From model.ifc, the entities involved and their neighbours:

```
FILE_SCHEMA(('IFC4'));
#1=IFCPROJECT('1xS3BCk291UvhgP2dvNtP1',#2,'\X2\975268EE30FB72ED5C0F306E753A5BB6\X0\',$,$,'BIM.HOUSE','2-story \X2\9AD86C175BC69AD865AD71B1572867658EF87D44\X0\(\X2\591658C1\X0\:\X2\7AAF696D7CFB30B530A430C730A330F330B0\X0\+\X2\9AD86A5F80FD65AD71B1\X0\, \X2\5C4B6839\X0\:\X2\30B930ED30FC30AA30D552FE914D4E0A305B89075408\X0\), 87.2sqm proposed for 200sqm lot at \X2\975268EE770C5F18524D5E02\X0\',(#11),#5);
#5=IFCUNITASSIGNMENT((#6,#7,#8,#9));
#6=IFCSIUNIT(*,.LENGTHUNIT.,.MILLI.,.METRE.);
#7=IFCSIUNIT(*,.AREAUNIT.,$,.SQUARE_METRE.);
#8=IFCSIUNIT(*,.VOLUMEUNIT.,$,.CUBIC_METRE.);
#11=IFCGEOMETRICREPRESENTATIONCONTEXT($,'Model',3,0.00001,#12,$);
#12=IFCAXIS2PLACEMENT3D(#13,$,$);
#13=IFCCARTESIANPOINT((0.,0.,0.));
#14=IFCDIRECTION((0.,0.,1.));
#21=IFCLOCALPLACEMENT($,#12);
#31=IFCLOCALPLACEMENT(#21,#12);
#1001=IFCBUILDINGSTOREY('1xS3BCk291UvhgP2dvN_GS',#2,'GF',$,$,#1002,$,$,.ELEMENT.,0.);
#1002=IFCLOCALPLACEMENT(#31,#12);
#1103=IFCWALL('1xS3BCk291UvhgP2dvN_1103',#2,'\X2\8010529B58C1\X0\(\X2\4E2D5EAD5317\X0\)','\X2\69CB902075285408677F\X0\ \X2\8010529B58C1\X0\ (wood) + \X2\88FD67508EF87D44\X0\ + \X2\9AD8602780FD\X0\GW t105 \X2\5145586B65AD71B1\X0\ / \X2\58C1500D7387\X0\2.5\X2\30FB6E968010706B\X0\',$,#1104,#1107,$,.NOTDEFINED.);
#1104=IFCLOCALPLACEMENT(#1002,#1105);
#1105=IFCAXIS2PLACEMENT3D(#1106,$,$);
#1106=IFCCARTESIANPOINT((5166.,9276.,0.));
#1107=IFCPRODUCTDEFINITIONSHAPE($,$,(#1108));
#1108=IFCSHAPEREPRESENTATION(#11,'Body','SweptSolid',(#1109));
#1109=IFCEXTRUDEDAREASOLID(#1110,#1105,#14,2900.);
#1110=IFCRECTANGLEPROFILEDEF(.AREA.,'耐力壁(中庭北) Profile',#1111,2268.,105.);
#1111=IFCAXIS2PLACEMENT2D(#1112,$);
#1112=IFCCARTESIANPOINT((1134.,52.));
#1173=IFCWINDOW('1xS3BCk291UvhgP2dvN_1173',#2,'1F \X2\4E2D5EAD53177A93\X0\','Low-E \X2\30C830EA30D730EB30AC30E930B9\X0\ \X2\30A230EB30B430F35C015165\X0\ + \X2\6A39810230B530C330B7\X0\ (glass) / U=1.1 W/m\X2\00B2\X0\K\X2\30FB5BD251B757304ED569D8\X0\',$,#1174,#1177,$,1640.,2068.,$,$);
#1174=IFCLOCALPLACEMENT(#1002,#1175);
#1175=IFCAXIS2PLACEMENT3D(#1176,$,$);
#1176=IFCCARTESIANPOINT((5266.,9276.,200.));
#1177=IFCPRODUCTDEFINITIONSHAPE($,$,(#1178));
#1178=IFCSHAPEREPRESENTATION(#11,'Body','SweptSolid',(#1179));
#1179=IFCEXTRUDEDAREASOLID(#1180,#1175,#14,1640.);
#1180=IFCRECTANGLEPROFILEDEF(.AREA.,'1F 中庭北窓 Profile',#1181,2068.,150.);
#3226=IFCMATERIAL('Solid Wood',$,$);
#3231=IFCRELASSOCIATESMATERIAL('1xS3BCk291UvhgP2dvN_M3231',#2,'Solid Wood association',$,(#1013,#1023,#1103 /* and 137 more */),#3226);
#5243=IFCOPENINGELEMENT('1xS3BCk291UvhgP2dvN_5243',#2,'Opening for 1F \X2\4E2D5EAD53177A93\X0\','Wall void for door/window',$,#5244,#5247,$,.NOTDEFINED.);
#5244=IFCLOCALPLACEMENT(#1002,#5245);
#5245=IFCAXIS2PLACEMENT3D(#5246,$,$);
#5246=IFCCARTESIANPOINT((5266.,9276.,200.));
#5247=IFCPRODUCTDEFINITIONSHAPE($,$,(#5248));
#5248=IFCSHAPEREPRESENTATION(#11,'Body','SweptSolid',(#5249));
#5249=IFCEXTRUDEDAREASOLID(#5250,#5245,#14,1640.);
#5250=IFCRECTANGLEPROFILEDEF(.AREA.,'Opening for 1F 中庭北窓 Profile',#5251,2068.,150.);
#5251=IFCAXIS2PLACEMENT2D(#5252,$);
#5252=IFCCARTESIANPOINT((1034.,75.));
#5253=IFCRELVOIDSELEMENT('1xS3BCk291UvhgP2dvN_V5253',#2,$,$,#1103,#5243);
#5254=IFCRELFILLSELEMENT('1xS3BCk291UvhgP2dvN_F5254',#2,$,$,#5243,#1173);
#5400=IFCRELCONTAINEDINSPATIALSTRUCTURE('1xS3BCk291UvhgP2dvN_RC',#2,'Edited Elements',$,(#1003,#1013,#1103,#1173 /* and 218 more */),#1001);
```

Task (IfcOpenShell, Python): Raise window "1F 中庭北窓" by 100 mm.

```python
import numpy as np
import ifcopenshell
import ifcopenshell.api.geometry
import ifcopenshell.util.placement
import ifcopenshell.util.unit

model = ifcopenshell.open("model.ifc")
unit_scale = ifcopenshell.util.unit.calculate_unit_scale(model)

window = model.by_guid("1xS3BCk291UvhgP2dvN_1173")
opening = window.FillsVoids[0].RelatingOpeningElement
dz = 0.1 / unit_scale

shift = np.array([0.0, 0.0, dz])
# The window is not placed relative to its opening, so move both.
for product in (opening, window):
    matrix = ifcopenshell.util.placement.get_local_placement(product.ObjectPlacement)
    matrix[:3, 3] += shift
    ifcopenshell.api.geometry.edit_object_placement(model, product=product, matrix=matrix, is_si=False)

print(f"moved by {dz * unit_scale:+.3f} m")

model.write("model_updated.ifc")
```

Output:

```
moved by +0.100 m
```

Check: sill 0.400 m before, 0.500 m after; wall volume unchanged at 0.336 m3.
